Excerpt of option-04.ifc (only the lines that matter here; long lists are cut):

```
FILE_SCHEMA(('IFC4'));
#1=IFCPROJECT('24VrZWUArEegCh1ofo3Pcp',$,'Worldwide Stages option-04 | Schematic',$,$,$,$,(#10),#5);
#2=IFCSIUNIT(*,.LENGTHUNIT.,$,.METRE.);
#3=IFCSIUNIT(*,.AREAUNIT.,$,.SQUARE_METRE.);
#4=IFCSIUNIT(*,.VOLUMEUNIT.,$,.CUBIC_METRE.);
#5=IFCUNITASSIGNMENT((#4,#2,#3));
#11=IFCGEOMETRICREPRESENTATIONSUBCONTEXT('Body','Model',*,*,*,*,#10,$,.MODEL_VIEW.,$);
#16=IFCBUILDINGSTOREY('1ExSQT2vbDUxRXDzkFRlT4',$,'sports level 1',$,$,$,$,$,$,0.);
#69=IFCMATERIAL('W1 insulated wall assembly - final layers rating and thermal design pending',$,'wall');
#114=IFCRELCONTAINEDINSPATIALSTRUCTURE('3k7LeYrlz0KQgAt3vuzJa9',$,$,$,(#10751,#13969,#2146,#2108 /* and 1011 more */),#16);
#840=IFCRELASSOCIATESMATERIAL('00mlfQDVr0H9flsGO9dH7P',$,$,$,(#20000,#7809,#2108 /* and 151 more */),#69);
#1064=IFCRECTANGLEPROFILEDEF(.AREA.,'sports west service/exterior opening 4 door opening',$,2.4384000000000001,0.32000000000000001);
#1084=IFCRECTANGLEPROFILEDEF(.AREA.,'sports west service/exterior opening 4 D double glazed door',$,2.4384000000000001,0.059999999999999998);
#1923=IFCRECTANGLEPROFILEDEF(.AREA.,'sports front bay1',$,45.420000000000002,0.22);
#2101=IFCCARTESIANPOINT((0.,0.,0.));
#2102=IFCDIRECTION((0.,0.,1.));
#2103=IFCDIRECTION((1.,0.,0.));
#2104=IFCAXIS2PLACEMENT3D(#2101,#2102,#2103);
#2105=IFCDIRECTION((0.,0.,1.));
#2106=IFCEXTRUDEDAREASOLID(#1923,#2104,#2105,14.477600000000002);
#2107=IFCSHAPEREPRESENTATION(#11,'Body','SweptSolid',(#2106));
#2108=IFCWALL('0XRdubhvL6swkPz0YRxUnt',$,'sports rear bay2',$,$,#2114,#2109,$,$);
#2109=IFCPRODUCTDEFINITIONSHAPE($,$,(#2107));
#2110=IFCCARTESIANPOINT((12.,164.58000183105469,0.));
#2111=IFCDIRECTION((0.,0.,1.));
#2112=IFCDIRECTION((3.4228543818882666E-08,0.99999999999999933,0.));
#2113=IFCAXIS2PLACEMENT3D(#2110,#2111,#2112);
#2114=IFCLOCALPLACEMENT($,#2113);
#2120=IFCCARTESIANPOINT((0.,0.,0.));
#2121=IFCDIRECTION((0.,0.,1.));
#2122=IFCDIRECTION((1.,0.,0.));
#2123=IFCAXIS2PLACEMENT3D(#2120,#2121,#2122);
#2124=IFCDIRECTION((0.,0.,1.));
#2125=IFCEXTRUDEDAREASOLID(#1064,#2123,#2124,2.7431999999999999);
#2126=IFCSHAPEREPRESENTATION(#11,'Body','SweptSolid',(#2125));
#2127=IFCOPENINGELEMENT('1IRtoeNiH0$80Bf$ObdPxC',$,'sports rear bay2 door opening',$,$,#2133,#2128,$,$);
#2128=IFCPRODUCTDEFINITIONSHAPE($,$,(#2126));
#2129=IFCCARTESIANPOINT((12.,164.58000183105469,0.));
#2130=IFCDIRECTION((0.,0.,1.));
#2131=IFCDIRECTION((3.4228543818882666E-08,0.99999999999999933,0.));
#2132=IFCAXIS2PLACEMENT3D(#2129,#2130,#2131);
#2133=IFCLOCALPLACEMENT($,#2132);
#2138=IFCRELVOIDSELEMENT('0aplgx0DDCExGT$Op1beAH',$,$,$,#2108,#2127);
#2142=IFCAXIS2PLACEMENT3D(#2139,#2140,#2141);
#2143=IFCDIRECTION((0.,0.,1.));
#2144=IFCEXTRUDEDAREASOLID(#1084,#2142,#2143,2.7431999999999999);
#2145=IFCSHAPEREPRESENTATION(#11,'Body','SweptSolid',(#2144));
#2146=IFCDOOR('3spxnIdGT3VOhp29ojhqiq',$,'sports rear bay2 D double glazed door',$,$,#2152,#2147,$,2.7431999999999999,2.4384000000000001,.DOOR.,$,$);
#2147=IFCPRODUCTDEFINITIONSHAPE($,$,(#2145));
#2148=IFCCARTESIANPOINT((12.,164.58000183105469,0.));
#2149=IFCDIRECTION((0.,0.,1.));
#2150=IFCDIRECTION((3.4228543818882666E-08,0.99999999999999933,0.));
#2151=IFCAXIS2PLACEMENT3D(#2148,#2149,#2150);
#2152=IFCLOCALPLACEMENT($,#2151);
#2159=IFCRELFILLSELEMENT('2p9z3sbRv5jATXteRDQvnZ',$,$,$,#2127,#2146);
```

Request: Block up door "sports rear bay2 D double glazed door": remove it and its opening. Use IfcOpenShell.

```python
import ifcopenshell
import ifcopenshell.api.feature
import ifcopenshell.api.root
import ifcopenshell.geom
import ifcopenshell.util.shape

model = ifcopenshell.open("option-04.ifc")
settings = ifcopenshell.geom.settings()


def volume(element):
    """Net volume in cubic metres, openings subtracted."""
    shape = ifcopenshell.geom.create_shape(settings, element)
    return ifcopenshell.util.shape.get_volume(shape.geometry)


door = model.by_id(2146)
opening = door.FillsVoids[0].RelatingOpeningElement
wall = opening.VoidsElements[0].RelatingBuildingElement
before = volume(wall)

ifcopenshell.api.root.remove_product(model, product=door)
ifcopenshell.api.feature.remove_feature(model, feature=opening)

after = volume(wall)

print(f"wall volume {before:.3f} -> {after:.3f} m3")

model.write("option-04_rev.ifc")
```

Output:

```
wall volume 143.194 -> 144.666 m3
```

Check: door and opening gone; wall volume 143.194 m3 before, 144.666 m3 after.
